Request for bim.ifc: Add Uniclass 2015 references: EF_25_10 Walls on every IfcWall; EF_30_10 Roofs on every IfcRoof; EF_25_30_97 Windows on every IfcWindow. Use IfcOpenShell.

First a look at what the model holds.

```python
import ifcopenshell

model = ifcopenshell.open("bim.ifc")
print(model.schema)
print("classifications:", [c.Name for c in model.by_type("IfcClassification")])
for ifc_class in ("IfcDoor", "IfcRoof", "IfcStair", "IfcWall", "IfcWindow"):
    print(ifc_class, len(model.by_type(ifc_class)))
```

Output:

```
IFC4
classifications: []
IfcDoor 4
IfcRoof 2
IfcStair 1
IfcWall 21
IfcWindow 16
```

```python
import ifcopenshell
import ifcopenshell.api.classification

model = ifcopenshell.open("bim.ifc")

system = ifcopenshell.api.classification.add_classification(model, classification="Uniclass 2015")

codes = {
    "IfcWall": ("EF_25_10", "Walls"),
    "IfcRoof": ("EF_30_10", "Roofs"),
    "IfcWindow": ("EF_25_30_97", "Windows"),
}
for ifc_class, (code, name) in codes.items():
    products = model.by_type(ifc_class)
    ifcopenshell.api.classification.add_reference(
        model, products=products, classification=system, identification=code, name=name
    )
    print(code, len(products))

model.write("bim-out.ifc")
```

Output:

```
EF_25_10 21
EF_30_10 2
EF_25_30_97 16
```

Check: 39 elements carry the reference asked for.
